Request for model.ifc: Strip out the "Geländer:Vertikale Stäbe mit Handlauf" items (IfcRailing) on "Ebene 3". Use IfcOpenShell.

First a look at what the model holds.

```python
import ifcopenshell
import ifcopenshell.util.element

model = ifcopenshell.open("model.ifc")
print(model.schema)
storey = next(s for s in model.by_type("IfcBuildingStorey") if s.Name == "Ebene 3")
railings = [e for e in ifcopenshell.util.element.get_decomposition(storey) if e.is_a("IfcRailing")]
seen = {}
for e in railings:
    element_type = ifcopenshell.util.element.get_type(e)
    name = element_type.Name if element_type not in (None, e) else None
    seen[name] = seen.get(name, 0) + 1
for name, count in sorted(seen.items(), key=str):
    print(count, "x", name)
```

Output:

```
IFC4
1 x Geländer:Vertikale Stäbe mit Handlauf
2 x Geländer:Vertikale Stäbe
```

```python
import ifcopenshell
import ifcopenshell.api.root
import ifcopenshell.util.element

model = ifcopenshell.open("model.ifc")

storey = next(s for s in model.by_type("IfcBuildingStorey") if s.Name == "Ebene 3")
railings = [e for e in ifcopenshell.util.element.get_decomposition(storey) if e.is_a("IfcRailing")]
targets = [e for e in railings if (t := ifcopenshell.util.element.get_type(e)) not in (None, e) and t.Name == "Geländer:Vertikale Stäbe mit Handlauf"]

for e in targets:
    ifcopenshell.api.root.remove_product(model, product=e)
print(len(targets), "removed")

model.write("model_rev.ifc")
```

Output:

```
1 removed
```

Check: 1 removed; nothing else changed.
